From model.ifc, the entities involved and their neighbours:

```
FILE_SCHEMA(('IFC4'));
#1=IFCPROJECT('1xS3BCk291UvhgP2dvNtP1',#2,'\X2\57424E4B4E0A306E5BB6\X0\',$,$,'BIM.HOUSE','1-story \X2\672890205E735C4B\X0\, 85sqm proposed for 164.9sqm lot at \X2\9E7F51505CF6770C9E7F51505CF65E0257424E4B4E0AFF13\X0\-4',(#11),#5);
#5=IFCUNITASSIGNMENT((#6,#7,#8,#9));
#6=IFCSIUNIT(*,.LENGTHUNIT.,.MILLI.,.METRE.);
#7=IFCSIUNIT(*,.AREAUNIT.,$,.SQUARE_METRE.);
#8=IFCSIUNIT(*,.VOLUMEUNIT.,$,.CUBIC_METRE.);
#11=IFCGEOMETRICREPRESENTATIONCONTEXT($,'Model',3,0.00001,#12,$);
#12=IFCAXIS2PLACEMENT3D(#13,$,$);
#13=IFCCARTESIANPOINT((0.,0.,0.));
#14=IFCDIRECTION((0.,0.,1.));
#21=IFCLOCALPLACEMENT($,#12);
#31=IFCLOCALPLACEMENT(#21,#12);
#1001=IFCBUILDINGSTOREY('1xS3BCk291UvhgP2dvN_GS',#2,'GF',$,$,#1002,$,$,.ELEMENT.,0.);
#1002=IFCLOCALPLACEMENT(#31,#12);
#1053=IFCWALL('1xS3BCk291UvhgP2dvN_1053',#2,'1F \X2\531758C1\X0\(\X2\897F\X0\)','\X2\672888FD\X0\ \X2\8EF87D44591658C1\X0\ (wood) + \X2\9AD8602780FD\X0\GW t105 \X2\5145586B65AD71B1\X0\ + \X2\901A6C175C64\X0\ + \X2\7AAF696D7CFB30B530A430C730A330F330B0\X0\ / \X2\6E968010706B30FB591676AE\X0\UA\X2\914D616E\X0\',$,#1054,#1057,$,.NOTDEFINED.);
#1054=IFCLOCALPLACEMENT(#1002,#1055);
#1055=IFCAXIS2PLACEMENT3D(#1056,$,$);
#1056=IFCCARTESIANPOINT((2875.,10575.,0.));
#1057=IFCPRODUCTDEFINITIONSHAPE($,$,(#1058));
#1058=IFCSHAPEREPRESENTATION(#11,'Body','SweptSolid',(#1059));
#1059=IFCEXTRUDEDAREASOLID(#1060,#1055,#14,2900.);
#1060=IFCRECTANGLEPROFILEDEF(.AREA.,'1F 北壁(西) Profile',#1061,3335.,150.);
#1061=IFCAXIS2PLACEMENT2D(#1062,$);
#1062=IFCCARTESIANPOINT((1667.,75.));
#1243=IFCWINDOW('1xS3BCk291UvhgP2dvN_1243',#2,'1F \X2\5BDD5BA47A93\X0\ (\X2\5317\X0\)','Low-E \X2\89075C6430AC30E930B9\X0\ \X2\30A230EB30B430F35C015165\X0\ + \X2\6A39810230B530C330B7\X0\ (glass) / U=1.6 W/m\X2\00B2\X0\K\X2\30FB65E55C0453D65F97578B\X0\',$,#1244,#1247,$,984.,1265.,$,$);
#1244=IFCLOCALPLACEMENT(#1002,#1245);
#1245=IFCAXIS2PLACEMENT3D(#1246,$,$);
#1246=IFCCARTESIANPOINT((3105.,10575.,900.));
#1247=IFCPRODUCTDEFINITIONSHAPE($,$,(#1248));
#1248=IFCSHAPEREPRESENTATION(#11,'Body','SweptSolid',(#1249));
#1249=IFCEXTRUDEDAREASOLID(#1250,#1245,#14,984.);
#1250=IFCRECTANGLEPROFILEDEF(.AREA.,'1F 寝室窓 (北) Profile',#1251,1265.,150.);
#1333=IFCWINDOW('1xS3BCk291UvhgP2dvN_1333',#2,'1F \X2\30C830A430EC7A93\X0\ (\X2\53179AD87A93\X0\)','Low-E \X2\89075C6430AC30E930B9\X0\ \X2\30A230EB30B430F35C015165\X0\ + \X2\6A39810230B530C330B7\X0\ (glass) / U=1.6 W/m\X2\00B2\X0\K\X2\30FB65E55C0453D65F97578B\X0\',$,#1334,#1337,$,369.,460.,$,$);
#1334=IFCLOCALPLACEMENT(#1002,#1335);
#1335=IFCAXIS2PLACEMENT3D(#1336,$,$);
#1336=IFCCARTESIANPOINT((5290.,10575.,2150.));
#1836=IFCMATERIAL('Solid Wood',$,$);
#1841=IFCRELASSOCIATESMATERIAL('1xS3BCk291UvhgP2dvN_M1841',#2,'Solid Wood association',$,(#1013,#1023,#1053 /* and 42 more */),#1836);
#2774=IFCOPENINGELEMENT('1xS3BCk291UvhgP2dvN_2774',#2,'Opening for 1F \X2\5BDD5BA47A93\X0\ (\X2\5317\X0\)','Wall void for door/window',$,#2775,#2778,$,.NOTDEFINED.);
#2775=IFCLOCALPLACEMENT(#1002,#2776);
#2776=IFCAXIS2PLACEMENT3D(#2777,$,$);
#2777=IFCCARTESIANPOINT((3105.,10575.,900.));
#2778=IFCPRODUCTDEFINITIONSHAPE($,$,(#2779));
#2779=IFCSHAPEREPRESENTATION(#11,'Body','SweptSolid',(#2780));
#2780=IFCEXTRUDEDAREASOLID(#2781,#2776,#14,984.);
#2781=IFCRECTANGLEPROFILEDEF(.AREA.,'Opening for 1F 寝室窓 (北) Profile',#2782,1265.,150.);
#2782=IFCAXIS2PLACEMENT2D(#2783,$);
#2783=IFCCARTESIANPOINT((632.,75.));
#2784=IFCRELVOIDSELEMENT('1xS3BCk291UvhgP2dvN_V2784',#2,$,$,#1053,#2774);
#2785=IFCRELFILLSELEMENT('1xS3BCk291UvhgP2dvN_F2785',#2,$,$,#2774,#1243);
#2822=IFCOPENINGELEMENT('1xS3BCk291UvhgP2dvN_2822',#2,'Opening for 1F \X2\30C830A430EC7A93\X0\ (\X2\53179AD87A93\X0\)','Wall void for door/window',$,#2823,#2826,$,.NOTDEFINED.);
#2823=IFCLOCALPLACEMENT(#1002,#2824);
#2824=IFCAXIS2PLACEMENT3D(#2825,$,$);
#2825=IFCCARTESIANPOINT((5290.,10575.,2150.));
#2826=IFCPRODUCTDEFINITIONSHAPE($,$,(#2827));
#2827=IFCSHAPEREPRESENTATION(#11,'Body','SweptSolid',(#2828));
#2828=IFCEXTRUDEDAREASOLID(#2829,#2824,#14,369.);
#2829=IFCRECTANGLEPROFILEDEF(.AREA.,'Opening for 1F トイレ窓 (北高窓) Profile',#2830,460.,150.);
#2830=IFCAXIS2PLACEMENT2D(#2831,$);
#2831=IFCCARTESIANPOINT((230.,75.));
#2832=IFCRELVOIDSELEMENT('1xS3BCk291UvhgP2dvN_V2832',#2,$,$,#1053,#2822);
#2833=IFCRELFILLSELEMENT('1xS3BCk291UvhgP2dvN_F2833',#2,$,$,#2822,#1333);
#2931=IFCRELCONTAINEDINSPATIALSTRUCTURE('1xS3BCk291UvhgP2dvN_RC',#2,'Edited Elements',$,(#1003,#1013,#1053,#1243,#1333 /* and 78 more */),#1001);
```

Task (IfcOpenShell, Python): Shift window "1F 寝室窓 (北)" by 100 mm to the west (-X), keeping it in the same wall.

```python
import ifcopenshell
import ifcopenshell.api.geometry
import ifcopenshell.util.placement

model = ifcopenshell.open("model.ifc")

window = model.by_guid("1xS3BCk291UvhgP2dvN_1243")
opening = window.FillsVoids[0].RelatingOpeningElement
wall = opening.VoidsElements[0].RelatingBuildingElement

wall_matrix = ifcopenshell.util.placement.get_local_placement(wall.ObjectPlacement)
shift = wall_matrix[:3, 0] * -100.0
before = ifcopenshell.util.placement.get_local_placement(window.ObjectPlacement)[:3, 3].copy()

# The window is not placed relative to its opening, so move both.
for product in (opening, window):
    matrix = ifcopenshell.util.placement.get_local_placement(product.ObjectPlacement)
    matrix[:3, 3] += shift
    ifcopenshell.api.geometry.edit_object_placement(model, product=product, matrix=matrix, is_si=False)

after = ifcopenshell.util.placement.get_local_placement(window.ObjectPlacement)[:3, 3]
print("window moved by", (after - before).round(3) + 0.0)

model.write("model_updated.ifc")
```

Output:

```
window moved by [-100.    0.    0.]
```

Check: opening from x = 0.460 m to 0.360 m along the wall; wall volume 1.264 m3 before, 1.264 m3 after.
